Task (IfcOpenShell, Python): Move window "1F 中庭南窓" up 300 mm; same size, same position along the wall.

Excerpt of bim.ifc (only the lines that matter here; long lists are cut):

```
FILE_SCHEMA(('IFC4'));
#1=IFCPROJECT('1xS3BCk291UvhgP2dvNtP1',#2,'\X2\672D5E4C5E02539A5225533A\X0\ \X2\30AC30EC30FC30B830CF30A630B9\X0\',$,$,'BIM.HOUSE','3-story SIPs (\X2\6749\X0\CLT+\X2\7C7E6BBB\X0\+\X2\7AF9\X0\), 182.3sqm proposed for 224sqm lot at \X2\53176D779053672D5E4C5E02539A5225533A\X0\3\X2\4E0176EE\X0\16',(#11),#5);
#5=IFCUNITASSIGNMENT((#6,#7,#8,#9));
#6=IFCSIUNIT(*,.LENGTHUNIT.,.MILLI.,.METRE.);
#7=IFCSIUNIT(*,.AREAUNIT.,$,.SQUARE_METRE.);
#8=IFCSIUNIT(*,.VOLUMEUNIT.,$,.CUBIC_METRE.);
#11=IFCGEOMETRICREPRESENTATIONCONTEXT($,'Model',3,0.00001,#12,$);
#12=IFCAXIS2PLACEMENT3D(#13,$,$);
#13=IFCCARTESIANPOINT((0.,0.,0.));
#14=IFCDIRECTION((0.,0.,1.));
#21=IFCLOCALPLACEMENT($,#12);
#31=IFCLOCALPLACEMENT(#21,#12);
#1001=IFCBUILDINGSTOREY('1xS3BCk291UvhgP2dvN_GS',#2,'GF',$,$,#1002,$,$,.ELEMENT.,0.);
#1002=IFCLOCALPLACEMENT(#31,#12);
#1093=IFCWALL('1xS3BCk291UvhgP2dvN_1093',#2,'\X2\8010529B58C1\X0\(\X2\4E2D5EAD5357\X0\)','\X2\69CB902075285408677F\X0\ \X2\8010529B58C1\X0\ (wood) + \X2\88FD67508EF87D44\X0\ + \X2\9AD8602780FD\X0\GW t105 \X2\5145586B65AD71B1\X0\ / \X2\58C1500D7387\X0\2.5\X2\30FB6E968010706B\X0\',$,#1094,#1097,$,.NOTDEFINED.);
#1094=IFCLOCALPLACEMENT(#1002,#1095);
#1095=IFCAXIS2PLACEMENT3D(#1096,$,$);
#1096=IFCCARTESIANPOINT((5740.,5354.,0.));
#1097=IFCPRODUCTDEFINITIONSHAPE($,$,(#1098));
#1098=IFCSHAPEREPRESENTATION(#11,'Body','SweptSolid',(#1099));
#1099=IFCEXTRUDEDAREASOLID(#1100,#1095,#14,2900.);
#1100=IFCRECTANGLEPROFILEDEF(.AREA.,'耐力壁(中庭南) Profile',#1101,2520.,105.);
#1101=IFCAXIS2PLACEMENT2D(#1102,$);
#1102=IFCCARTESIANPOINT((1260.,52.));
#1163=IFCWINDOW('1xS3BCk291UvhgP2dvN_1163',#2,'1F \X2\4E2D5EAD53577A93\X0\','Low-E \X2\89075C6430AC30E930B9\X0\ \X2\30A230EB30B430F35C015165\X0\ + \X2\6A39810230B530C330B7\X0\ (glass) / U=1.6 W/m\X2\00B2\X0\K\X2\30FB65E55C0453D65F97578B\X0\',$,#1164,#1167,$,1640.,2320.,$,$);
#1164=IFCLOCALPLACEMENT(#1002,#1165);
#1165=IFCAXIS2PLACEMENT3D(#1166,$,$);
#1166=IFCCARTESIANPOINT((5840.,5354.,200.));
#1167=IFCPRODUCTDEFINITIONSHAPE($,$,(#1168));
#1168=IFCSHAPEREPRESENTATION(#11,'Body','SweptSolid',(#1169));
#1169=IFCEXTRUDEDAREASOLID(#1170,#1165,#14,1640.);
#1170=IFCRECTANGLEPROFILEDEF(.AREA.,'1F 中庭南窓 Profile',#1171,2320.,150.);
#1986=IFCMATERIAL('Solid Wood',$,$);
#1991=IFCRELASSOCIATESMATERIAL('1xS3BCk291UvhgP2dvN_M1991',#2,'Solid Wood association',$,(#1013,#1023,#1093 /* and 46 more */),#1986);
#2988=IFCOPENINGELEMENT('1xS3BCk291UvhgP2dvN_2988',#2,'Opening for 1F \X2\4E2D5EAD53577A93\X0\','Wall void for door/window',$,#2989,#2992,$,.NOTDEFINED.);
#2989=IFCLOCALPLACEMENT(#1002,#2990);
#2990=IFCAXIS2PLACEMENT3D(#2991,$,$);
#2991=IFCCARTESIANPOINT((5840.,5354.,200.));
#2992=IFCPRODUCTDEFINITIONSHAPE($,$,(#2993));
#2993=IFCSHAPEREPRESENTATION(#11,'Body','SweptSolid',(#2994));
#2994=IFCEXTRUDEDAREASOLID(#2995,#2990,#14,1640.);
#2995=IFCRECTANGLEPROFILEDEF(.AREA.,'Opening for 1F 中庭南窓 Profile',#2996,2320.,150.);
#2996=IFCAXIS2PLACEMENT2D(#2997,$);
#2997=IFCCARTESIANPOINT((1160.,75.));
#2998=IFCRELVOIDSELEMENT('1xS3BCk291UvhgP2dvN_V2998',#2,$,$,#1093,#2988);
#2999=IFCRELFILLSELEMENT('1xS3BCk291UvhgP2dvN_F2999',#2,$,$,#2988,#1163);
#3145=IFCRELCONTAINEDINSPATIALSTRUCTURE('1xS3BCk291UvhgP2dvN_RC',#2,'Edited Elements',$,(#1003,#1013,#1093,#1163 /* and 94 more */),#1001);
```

```python
import numpy as np
import ifcopenshell
import ifcopenshell.api.geometry
import ifcopenshell.util.placement
import ifcopenshell.util.unit

model = ifcopenshell.open("bim.ifc")
unit_scale = ifcopenshell.util.unit.calculate_unit_scale(model)

window = model.by_guid("1xS3BCk291UvhgP2dvN_1163")
opening = window.FillsVoids[0].RelatingOpeningElement
dz = 300.0

shift = np.array([0.0, 0.0, dz])
# The window is not placed relative to its opening, so move both.
for product in (opening, window):
    matrix = ifcopenshell.util.placement.get_local_placement(product.ObjectPlacement)
    matrix[:3, 3] += shift
    ifcopenshell.api.geometry.edit_object_placement(model, product=product, matrix=matrix, is_si=False)

print(f"moved by {dz * unit_scale:+.3f} m")

model.write("bim_rev.ifc")
```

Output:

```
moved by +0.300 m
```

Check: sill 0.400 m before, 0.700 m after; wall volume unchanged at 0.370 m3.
